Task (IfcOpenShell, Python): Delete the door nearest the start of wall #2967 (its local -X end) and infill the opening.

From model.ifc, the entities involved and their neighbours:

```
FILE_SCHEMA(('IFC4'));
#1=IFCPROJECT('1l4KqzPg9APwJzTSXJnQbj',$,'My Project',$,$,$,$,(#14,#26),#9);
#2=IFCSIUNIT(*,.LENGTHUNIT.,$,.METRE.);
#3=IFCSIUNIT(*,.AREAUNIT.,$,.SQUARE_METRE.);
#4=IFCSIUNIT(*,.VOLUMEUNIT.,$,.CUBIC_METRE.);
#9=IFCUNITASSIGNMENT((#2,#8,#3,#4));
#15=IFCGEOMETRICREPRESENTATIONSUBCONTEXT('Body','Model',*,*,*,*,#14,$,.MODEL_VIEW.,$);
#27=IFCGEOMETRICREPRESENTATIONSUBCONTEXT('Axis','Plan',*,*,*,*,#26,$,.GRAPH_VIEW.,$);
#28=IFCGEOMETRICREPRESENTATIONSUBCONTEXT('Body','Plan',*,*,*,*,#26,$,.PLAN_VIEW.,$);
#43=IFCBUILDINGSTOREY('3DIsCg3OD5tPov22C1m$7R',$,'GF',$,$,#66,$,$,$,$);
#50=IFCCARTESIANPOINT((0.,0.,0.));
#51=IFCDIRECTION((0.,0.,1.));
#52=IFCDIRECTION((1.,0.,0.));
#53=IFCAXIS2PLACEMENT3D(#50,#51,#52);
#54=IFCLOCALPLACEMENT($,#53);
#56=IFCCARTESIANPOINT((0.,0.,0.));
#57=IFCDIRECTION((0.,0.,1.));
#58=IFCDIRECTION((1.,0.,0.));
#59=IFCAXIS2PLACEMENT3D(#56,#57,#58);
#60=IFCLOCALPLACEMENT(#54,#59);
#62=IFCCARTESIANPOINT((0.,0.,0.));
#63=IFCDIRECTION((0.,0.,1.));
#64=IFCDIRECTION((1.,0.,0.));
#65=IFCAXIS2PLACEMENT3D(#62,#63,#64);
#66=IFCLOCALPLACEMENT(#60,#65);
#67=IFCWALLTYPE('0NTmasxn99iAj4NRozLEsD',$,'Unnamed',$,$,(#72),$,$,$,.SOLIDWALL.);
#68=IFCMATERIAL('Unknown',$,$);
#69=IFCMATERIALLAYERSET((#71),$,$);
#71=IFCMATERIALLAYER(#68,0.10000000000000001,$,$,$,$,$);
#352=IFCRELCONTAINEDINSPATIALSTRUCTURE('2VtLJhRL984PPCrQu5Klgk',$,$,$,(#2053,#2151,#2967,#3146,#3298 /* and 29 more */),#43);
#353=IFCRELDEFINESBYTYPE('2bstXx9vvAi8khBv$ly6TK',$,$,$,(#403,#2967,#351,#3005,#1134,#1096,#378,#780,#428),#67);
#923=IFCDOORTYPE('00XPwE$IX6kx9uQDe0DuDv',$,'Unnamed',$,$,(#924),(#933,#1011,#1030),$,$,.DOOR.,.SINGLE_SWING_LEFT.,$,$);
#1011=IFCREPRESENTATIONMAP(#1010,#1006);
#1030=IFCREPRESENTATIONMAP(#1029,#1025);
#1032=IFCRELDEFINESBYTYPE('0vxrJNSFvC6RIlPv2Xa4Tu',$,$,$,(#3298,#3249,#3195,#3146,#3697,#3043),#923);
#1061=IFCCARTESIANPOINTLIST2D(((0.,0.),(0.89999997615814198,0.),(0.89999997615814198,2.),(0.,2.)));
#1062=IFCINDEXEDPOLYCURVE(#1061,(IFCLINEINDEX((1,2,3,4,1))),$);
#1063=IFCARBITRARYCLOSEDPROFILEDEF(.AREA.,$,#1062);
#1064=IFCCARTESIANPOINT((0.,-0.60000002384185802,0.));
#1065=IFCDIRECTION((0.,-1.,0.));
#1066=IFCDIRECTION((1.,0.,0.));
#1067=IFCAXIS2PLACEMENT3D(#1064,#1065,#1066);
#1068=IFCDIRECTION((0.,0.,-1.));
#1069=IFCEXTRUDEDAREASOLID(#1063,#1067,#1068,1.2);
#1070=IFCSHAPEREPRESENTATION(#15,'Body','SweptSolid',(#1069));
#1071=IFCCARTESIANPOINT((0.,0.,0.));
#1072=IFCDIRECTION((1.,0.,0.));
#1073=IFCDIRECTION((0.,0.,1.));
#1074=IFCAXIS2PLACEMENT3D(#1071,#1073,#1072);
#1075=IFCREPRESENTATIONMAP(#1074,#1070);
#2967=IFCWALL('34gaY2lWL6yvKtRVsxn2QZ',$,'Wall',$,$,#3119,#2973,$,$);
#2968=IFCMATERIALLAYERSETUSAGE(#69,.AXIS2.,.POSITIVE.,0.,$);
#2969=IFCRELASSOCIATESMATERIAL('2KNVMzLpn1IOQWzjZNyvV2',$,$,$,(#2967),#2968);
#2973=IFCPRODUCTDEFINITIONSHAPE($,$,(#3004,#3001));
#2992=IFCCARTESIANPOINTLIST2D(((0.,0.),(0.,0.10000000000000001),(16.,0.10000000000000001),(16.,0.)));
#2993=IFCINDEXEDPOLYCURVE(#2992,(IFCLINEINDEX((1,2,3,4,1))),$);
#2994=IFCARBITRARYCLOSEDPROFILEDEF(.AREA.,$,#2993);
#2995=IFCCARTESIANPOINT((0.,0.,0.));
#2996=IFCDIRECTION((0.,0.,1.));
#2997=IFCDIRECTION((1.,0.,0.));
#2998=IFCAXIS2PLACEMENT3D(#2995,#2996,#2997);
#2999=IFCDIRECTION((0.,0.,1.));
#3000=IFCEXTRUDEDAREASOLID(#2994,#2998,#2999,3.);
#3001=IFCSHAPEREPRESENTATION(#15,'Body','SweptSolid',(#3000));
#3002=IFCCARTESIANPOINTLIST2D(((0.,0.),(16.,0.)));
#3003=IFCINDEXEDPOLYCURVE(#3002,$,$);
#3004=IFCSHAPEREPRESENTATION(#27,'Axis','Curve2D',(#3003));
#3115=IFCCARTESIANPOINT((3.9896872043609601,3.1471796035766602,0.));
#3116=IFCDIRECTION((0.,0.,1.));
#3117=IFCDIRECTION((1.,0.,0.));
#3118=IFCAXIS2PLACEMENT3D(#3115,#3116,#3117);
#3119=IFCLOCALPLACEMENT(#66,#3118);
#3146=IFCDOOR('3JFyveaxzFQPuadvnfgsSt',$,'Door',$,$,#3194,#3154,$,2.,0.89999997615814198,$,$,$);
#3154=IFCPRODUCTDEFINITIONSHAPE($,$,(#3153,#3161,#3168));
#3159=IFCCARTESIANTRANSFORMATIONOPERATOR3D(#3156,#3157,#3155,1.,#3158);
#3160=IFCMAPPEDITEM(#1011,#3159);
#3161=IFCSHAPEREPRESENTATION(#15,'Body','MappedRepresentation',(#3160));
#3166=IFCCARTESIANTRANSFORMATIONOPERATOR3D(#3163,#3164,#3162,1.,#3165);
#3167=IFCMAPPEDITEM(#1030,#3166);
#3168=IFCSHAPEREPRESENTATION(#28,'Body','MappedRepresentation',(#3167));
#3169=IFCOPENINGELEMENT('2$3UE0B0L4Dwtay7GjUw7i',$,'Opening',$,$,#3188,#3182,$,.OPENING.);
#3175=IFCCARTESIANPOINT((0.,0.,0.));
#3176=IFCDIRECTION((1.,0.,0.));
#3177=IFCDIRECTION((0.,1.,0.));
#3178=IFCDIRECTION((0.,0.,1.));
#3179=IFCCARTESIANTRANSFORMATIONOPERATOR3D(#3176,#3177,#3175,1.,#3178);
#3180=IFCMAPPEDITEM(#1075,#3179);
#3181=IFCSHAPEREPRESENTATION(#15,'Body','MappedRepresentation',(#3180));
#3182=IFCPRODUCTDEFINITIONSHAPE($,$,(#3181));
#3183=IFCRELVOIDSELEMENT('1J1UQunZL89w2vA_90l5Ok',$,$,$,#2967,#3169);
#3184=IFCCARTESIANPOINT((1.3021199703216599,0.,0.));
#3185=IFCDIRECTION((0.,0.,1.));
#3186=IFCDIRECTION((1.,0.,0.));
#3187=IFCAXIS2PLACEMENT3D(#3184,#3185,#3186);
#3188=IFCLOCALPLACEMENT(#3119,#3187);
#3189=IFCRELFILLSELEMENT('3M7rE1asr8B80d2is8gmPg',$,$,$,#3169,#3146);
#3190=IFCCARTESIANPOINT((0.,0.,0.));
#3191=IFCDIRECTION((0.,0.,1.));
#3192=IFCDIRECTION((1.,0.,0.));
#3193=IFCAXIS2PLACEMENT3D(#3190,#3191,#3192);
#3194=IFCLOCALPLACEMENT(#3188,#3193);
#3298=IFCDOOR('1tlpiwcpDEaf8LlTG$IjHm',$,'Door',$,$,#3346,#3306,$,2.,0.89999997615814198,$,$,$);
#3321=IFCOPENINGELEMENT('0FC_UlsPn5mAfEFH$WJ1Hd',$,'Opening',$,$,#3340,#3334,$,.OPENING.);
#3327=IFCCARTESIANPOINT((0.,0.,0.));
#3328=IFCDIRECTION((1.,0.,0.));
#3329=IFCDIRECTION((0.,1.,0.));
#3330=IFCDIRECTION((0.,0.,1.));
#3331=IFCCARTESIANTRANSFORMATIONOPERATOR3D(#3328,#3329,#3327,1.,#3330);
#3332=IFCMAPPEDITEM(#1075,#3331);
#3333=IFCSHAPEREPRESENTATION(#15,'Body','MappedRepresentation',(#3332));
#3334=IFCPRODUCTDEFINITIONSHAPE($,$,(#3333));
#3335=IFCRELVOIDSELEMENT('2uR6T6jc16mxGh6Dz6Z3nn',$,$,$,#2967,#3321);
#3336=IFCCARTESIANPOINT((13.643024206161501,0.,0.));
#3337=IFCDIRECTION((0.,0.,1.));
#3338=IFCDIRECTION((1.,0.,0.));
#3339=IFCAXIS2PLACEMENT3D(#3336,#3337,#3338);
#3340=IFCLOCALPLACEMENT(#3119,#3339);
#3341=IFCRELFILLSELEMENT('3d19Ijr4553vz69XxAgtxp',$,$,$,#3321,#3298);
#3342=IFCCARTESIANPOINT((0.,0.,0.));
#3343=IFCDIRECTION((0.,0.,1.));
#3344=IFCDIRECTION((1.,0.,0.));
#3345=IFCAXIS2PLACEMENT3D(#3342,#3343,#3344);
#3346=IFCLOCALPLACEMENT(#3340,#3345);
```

```python
import ifcopenshell
import ifcopenshell.api.feature
import ifcopenshell.api.root
import ifcopenshell.geom
import ifcopenshell.util.shape

model = ifcopenshell.open("model.ifc")
settings = ifcopenshell.geom.settings()


def volume(element):
    """Net volume in cubic metres, openings subtracted."""
    shape = ifcopenshell.geom.create_shape(settings, element)
    return ifcopenshell.util.shape.get_volume(shape.geometry)


door = model.by_guid("3JFyveaxzFQPuadvnfgsSt")
opening = door.FillsVoids[0].RelatingOpeningElement
wall = opening.VoidsElements[0].RelatingBuildingElement
before = volume(wall)

ifcopenshell.api.root.remove_product(model, product=door)
ifcopenshell.api.feature.remove_feature(model, feature=opening)

after = volume(wall)

print(f"wall volume {before:.3f} -> {after:.3f} m3")

model.write("model_updated.ifc")
```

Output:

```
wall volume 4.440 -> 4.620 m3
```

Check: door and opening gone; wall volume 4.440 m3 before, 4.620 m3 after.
